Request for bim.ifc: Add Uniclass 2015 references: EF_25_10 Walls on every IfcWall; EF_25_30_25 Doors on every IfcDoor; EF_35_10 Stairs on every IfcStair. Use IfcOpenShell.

First a look at what the model holds.

```python
import ifcopenshell

model = ifcopenshell.open("bim.ifc")
print(model.schema)
print("classifications:", [c.Name for c in model.by_type("IfcClassification")])
for ifc_class in ("IfcDoor", "IfcRoof", "IfcStair", "IfcWall", "IfcWindow"):
    print(ifc_class, len(model.by_type(ifc_class)))
```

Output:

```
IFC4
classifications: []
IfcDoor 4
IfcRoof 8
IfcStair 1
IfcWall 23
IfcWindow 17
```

```python
import ifcopenshell
import ifcopenshell.api.classification

model = ifcopenshell.open("bim.ifc")

system = ifcopenshell.api.classification.add_classification(model, classification="Uniclass 2015")

codes = {
    "IfcWall": ("EF_25_10", "Walls"),
    "IfcDoor": ("EF_25_30_25", "Doors"),
    "IfcStair": ("EF_35_10", "Stairs"),
}
for ifc_class, (code, name) in codes.items():
    products = model.by_type(ifc_class)
    ifcopenshell.api.classification.add_reference(
        model, products=products, classification=system, identification=code, name=name
    )
    print(code, len(products))

model.write("bim_rev.ifc")
```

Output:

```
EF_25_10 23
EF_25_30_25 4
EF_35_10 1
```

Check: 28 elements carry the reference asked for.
